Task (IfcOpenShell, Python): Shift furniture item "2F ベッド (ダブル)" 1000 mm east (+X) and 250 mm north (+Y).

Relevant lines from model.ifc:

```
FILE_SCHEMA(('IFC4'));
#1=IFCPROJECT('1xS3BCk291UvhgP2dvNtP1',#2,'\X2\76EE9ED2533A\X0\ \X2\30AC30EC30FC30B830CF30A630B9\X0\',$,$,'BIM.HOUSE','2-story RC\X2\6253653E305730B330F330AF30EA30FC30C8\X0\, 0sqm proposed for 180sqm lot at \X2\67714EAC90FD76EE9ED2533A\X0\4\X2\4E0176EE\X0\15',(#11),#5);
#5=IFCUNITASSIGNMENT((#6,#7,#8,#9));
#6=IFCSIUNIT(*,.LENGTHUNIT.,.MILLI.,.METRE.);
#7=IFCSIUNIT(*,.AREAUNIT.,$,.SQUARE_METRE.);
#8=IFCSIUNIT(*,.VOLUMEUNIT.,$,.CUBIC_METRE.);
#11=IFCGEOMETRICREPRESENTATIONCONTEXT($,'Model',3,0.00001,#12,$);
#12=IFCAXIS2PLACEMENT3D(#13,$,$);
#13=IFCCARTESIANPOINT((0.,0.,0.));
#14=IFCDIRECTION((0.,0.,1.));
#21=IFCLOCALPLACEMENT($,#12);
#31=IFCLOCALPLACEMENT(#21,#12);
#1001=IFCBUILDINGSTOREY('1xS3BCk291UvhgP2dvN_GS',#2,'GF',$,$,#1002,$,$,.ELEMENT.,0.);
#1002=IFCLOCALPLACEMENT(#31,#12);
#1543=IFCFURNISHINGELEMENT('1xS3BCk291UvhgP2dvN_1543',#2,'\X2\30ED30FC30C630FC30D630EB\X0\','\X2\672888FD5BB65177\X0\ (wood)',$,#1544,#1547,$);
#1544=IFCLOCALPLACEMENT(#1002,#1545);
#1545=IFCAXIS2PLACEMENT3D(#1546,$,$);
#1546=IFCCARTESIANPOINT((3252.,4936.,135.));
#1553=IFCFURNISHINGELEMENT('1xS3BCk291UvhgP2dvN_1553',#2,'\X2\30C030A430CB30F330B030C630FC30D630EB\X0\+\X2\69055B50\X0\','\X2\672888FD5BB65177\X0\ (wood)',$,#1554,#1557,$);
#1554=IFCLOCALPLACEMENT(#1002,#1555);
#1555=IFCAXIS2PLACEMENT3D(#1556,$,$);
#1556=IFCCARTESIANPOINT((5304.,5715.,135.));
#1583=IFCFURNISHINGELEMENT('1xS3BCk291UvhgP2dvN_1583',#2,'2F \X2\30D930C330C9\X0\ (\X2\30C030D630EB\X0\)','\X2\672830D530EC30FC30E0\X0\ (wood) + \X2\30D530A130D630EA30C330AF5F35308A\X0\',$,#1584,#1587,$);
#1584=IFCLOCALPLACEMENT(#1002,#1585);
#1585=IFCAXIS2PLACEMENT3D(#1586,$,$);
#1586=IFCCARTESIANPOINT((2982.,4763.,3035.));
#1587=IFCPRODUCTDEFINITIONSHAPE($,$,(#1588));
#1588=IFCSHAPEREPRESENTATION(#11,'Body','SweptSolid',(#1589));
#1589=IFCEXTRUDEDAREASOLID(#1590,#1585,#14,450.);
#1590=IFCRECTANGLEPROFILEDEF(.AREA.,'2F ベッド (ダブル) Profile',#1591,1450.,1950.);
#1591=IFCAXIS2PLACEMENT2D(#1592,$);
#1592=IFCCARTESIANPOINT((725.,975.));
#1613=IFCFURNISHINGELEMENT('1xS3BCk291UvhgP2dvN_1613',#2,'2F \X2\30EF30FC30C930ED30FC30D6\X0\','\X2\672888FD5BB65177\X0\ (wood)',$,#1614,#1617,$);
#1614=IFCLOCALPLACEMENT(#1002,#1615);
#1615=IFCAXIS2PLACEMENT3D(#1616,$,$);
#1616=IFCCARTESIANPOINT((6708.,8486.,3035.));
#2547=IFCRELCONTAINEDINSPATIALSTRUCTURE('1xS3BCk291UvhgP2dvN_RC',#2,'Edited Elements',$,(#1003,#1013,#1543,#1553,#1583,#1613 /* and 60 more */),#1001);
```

```python
import ifcopenshell
import ifcopenshell.api.geometry
import ifcopenshell.util.placement
import ifcopenshell.util.unit

model = ifcopenshell.open("model.ifc")
unit_scale = ifcopenshell.util.unit.calculate_unit_scale(model)

item = model.by_guid("1xS3BCk291UvhgP2dvN_1583")
matrix = ifcopenshell.util.placement.get_local_placement(item.ObjectPlacement)
matrix[0, 3] += 1 / unit_scale
matrix[1, 3] += 0.25 / unit_scale
ifcopenshell.api.geometry.edit_object_placement(model, product=item, matrix=matrix, is_si=False)

print(ifcopenshell.util.placement.get_local_placement(item.ObjectPlacement).round(3) + 0.0)

model.write("model_rev.ifc")
```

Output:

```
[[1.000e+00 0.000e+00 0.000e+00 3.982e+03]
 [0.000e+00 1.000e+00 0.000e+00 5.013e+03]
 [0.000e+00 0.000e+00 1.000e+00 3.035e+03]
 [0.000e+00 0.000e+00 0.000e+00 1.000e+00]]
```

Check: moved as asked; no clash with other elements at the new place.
